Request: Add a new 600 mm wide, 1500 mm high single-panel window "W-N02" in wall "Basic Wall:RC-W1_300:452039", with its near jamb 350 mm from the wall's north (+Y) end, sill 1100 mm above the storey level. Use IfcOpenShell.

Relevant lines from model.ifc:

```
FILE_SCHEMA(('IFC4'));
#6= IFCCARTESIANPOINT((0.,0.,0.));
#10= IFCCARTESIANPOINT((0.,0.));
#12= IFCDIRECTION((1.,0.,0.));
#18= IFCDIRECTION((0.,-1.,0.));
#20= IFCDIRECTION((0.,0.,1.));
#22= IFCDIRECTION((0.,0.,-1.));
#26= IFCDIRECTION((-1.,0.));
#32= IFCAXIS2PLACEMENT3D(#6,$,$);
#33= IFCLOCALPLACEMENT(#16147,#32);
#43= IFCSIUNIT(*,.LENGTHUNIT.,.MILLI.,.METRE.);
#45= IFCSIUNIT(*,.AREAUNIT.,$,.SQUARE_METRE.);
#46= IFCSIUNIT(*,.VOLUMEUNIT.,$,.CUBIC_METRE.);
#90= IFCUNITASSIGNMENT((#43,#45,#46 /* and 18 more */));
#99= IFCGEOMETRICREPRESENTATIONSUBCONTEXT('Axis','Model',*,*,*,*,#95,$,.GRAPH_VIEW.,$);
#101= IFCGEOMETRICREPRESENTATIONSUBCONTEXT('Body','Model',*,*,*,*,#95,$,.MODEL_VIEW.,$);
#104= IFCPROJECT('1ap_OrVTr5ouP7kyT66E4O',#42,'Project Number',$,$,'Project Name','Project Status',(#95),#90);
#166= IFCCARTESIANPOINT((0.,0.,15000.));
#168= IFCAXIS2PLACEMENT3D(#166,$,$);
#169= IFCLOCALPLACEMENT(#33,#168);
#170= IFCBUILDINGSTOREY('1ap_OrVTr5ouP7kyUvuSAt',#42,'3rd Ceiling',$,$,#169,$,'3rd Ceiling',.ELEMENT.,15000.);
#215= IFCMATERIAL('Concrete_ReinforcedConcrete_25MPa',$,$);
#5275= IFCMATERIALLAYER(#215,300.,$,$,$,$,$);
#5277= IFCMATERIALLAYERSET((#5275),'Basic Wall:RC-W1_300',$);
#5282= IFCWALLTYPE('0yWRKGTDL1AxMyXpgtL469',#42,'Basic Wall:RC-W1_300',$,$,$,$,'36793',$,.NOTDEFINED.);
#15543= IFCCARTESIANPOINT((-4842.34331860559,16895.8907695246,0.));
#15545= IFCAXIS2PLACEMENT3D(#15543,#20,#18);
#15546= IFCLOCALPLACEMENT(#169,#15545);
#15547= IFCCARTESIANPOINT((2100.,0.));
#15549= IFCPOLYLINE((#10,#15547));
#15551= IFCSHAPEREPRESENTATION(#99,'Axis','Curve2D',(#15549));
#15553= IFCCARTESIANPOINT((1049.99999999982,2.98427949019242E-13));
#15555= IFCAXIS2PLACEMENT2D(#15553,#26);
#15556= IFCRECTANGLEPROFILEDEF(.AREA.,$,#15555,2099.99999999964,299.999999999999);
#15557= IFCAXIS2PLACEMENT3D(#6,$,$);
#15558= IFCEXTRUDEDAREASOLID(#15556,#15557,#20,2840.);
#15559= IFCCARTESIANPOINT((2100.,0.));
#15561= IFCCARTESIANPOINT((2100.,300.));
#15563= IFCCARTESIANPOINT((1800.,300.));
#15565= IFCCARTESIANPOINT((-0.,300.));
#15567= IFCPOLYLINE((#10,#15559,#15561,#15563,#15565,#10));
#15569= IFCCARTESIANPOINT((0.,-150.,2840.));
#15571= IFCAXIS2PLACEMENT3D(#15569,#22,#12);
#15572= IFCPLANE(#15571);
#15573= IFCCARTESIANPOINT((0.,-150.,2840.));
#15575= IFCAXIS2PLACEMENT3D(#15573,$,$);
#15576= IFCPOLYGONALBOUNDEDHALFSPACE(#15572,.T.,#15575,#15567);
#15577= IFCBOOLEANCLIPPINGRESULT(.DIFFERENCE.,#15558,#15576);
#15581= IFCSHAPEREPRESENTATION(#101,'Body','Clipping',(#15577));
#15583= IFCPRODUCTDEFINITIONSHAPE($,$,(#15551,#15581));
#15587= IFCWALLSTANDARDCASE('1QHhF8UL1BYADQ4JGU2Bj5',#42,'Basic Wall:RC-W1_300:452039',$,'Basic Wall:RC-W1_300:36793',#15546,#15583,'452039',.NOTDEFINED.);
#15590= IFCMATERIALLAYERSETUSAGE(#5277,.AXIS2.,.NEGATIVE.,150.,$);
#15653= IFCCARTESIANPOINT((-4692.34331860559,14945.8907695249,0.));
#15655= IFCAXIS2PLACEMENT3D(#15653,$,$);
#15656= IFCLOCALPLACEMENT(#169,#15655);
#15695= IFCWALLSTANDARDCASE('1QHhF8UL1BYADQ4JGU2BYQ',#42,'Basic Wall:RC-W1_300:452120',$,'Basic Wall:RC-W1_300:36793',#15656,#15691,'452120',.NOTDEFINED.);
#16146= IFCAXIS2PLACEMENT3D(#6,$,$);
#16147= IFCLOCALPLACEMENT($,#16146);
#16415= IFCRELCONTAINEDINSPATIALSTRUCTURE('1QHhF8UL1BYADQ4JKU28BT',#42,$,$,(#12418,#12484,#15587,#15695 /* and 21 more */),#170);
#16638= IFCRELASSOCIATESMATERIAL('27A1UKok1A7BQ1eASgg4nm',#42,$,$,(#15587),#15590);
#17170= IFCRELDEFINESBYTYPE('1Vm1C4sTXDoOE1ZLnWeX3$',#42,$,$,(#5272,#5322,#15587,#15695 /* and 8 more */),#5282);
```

```python
import numpy as np
import ifcopenshell
import ifcopenshell.api.feature
import ifcopenshell.api.geometry
import ifcopenshell.api.root
import ifcopenshell.api.spatial
import ifcopenshell.geom
import ifcopenshell.util.element
import ifcopenshell.util.placement
import ifcopenshell.util.representation
import ifcopenshell.util.shape
import ifcopenshell.util.unit

model = ifcopenshell.open("model.ifc")
unit_scale = ifcopenshell.util.unit.calculate_unit_scale(model)
settings = ifcopenshell.geom.settings()


def volume(element):
    """Net volume in cubic metres, openings subtracted."""
    shape = ifcopenshell.geom.create_shape(settings, element)
    return ifcopenshell.util.shape.get_volume(shape.geometry)


wall = model.by_id(15587)
storey = ifcopenshell.util.element.get_container(wall, ifc_class="IfcBuildingStorey")
context = ifcopenshell.util.representation.get_context(model, "Model", "Body", "MODEL_VIEW")
before = volume(wall)

width, height, from_end, sill = 0.6, 1.5, 0.35, 1.1  # metres

# The wall runs along its own X axis, and the end named is its -X end.
wall_shape = ifcopenshell.geom.create_shape(settings, wall)
x, y, z = ifcopenshell.util.shape.get_vertices(wall_shape.geometry).T
start = x.min() + from_end
face, thickness = float(y.min()), float(y.max() - y.min())
wall_matrix = ifcopenshell.util.placement.get_local_placement(wall.ObjectPlacement)
level = ifcopenshell.util.placement.get_local_placement(storey.ObjectPlacement)[2, 3]


def in_wall(x, y):
    """Placement at x, y metres in the wall's axes, at sill height."""
    matrix = wall_matrix.copy()
    matrix[:, 3] = wall_matrix @ np.array([x / unit_scale, y / unit_scale, 0.0, 1.0])
    matrix[2, 3] = level + sill / unit_scale
    return matrix


# Opening: a box that overshoots both wall faces by 50 mm.
opening = ifcopenshell.api.root.create_entity(model, ifc_class="IfcOpeningElement", predefined_type="OPENING")
box = ifcopenshell.api.geometry.add_wall_representation(
    model, context=context, length=width, height=height, thickness=thickness + 0.1
)
ifcopenshell.api.geometry.assign_representation(model, product=opening, representation=box)
ifcopenshell.api.geometry.edit_object_placement(model, product=opening, matrix=in_wall(start, face - 0.05), is_si=False)
ifcopenshell.api.feature.add_feature(model, feature=opening, element=wall)

window = ifcopenshell.api.root.create_entity(model, ifc_class="IfcWindow", name="W-N02", predefined_type="WINDOW")
window.OverallWidth, window.OverallHeight = width / unit_scale, height / unit_scale
window.PartitioningType = "SINGLE_PANEL"
body = ifcopenshell.api.geometry.add_window_representation(
    model,
    context=context,
    overall_width=window.OverallWidth,
    overall_height=window.OverallHeight,
    partition_type="SINGLE_PANEL",
)
ifcopenshell.api.geometry.assign_representation(model, product=window, representation=body)
ifcopenshell.api.spatial.assign_container(model, products=[window], relating_structure=storey)
ifcopenshell.api.feature.add_filling(model, opening=opening, element=window)

# Centre the window in the wall's thickness.
ifcopenshell.api.geometry.edit_object_placement(model, product=window, matrix=in_wall(start, face), is_si=False)
window_shape = ifcopenshell.geom.create_shape(settings, window)
depth = ifcopenshell.util.shape.get_vertices(window_shape.geometry)[:, 1]
offset = face + thickness / 2 - (depth.min() + depth.max()) / 2
ifcopenshell.api.geometry.edit_object_placement(model, product=window, matrix=in_wall(start, offset), is_si=False)

after = volume(wall)

print(f"wall volume {before:.3f} -> {after:.3f} m3")

model.write("model_updated.ifc")
```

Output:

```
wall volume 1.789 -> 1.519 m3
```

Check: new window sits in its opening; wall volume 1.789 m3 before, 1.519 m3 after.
